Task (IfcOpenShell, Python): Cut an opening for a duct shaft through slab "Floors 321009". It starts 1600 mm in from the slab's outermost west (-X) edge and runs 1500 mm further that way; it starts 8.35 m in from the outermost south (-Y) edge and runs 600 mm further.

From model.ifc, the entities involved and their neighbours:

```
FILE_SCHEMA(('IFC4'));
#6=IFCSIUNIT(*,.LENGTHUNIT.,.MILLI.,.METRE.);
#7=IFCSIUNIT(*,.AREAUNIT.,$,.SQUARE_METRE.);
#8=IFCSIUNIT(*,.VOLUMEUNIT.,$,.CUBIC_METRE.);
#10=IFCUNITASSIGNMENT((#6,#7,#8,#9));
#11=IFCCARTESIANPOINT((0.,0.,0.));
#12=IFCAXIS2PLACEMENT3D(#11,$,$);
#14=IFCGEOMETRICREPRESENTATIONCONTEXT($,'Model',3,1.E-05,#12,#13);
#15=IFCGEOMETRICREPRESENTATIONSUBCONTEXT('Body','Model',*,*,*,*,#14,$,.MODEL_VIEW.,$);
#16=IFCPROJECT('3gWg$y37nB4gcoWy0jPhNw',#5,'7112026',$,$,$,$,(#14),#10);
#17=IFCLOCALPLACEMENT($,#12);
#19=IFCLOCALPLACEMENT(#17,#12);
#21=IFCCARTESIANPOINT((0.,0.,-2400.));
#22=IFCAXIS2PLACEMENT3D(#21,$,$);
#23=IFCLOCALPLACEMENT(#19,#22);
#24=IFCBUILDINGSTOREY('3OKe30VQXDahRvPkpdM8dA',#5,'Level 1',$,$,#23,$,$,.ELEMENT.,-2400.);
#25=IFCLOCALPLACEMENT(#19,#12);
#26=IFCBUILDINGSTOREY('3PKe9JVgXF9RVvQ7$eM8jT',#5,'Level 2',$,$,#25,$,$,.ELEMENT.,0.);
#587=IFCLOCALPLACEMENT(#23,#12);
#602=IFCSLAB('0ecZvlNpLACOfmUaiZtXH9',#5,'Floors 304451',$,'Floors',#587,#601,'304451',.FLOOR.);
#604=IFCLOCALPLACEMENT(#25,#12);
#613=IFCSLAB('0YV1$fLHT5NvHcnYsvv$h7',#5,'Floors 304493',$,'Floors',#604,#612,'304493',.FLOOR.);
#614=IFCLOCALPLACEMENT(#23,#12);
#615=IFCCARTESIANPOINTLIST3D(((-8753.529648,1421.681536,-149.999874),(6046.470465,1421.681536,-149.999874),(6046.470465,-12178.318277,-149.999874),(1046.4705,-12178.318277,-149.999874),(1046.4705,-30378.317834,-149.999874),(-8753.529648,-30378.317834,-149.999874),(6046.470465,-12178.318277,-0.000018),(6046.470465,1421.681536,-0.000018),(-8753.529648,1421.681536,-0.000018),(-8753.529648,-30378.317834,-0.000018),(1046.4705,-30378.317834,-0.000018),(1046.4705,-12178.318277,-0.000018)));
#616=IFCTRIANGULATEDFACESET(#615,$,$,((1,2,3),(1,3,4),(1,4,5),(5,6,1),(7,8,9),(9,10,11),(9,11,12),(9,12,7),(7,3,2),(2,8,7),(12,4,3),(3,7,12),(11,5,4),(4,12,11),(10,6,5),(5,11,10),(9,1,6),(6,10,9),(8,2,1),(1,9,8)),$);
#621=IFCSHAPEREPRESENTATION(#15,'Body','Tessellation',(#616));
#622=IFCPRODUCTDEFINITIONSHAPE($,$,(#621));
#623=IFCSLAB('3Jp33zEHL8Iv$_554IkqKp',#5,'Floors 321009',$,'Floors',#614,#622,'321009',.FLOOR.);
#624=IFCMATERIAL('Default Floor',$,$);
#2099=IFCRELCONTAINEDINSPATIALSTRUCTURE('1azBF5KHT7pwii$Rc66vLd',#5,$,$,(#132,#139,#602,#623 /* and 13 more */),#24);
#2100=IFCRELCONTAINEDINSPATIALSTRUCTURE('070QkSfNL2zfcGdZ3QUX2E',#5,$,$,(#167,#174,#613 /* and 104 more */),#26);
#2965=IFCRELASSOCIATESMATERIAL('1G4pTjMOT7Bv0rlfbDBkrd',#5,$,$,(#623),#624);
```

```python
import numpy as np
import ifcopenshell
import ifcopenshell.api.feature
import ifcopenshell.api.geometry
import ifcopenshell.api.root
import ifcopenshell.geom
import ifcopenshell.util.placement
import ifcopenshell.util.representation
import ifcopenshell.util.shape
import ifcopenshell.util.unit

model = ifcopenshell.open("model.ifc")
unit_scale = ifcopenshell.util.unit.calculate_unit_scale(model)
settings = ifcopenshell.geom.settings()


def volume(element):
    """Net volume in cubic metres, openings subtracted."""
    shape = ifcopenshell.geom.create_shape(settings, element)
    return ifcopenshell.util.shape.get_volume(shape.geometry)


slab = model.by_id(623)
before = volume(slab)

# Extent in the slab's own axes, in metres. The edges named are its -X and -Y sides.
slab_shape = ifcopenshell.geom.create_shape(settings, slab)
vertices = ifcopenshell.util.shape.get_vertices(slab_shape.geometry)
x_min, y_min, bottom = vertices.min(axis=0)
top = vertices[:, 2].max()

opening = ifcopenshell.api.root.create_entity(model, ifc_class="IfcOpeningElement", name="Duct shaft opening", predefined_type="OPENING")
context = ifcopenshell.util.representation.get_context(model, "Model", "Body", "MODEL_VIEW")
width, depth = 1.5, 0.6
outline = [(0.0, 0.0), (width, 0.0), (width, depth), (0.0, depth), (0.0, 0.0)]
# Overshoot both faces by 50 mm so the cut is clean.
shape = ifcopenshell.api.geometry.add_slab_representation(
    model, context=context, depth=top - bottom + 0.1, polyline=outline
)
ifcopenshell.api.geometry.assign_representation(model, product=opening, representation=shape)

matrix = ifcopenshell.util.placement.get_local_placement(slab.ObjectPlacement)
matrix[:, 3] = matrix @ np.append(np.array([x_min + 1.6, y_min + 8.35, bottom - 0.05]) / unit_scale, 1.0)
ifcopenshell.api.geometry.edit_object_placement(model, product=opening, matrix=matrix, is_si=False)
ifcopenshell.api.feature.add_feature(model, feature=opening, element=slab)

after = volume(slab)

print(f"slab volume {before:.3f} -> {after:.3f} m3")

model.write("model-out.ifc")
```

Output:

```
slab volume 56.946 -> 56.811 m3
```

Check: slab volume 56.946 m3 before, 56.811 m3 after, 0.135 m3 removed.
